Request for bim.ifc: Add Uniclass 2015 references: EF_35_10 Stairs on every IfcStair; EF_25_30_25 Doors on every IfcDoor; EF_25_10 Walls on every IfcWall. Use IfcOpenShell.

First a look at what the model holds.

```python
import ifcopenshell

model = ifcopenshell.open("bim.ifc")
print(model.schema)
print("classifications:", [c.Name for c in model.by_type("IfcClassification")])
for ifc_class in ("IfcDoor", "IfcRoof", "IfcStair", "IfcWall", "IfcWindow"):
    print(ifc_class, len(model.by_type(ifc_class)))
```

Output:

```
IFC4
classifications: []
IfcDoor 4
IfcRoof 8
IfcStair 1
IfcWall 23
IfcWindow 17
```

```python
import ifcopenshell
import ifcopenshell.api.classification

model = ifcopenshell.open("bim.ifc")

system = ifcopenshell.api.classification.add_classification(model, classification="Uniclass 2015")

codes = {
    "IfcStair": ("EF_35_10", "Stairs"),
    "IfcDoor": ("EF_25_30_25", "Doors"),
    "IfcWall": ("EF_25_10", "Walls"),
}
for ifc_class, (code, name) in codes.items():
    products = model.by_type(ifc_class)
    ifcopenshell.api.classification.add_reference(
        model, products=products, classification=system, identification=code, name=name
    )
    print(code, len(products))

model.write("bim_v2.ifc")
```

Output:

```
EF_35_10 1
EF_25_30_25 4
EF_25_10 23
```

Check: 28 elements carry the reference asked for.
